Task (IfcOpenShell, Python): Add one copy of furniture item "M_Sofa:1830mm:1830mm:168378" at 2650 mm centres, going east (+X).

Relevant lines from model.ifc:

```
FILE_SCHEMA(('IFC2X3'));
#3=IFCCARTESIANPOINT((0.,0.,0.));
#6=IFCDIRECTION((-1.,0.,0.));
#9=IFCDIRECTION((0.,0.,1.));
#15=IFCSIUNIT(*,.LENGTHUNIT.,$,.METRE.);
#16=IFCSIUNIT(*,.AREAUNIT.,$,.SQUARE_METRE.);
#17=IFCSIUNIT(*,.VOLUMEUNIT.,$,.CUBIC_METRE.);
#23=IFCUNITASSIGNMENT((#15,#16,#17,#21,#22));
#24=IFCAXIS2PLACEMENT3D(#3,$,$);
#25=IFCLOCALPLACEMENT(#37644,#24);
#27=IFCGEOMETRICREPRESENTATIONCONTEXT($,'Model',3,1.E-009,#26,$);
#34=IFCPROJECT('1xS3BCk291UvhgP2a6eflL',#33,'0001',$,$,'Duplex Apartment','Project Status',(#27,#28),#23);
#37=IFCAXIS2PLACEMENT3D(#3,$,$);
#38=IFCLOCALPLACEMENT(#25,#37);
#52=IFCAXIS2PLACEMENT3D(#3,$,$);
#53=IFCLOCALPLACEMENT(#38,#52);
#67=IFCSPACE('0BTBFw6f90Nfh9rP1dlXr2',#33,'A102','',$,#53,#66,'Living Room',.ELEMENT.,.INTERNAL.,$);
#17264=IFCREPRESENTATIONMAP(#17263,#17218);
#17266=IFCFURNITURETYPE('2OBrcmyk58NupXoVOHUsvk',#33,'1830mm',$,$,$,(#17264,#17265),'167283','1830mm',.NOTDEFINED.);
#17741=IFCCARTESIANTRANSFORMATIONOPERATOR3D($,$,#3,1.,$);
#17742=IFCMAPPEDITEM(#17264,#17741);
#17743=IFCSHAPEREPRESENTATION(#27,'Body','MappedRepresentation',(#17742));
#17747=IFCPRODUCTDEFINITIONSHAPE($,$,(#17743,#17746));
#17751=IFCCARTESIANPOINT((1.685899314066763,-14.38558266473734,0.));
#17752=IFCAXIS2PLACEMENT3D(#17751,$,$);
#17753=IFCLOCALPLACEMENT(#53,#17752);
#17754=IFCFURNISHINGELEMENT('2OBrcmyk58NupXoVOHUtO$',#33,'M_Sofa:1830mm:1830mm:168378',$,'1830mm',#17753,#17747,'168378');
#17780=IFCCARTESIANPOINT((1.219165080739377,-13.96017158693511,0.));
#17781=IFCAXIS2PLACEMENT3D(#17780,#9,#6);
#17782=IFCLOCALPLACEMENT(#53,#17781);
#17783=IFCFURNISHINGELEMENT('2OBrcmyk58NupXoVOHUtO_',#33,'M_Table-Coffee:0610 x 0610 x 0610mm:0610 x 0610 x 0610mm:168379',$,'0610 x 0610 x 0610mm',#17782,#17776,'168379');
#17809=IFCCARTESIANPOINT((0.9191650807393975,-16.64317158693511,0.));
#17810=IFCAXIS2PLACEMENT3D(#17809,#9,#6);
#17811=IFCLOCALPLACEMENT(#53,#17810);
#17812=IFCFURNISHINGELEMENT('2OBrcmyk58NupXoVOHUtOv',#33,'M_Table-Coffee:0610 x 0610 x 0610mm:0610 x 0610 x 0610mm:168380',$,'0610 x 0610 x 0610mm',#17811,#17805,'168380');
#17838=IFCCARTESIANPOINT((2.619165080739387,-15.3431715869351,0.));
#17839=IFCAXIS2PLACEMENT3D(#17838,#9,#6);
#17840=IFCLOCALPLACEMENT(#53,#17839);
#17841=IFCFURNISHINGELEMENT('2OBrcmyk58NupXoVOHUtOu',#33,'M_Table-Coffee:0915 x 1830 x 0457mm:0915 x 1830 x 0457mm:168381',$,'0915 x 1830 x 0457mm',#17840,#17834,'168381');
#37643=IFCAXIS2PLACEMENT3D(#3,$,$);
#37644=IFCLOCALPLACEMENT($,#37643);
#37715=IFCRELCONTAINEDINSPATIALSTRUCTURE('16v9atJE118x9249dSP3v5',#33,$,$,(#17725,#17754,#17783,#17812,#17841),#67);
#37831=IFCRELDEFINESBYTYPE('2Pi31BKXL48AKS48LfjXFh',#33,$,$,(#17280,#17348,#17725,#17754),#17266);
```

```python
import numpy as np
import ifcopenshell
import ifcopenshell.api.geometry
import ifcopenshell.api.root
import ifcopenshell.util.element
import ifcopenshell.util.placement

model = ifcopenshell.open("model.ifc")


def reuse_history(source, copy):
    """copy_class also copies each property set's owner history, people and application; keep the originals."""
    for rel in copy.IsDefinedBy:
        if rel.is_a("IfcRelDefinesByProperties") and (history := rel.RelatingPropertyDefinition.OwnerHistory):
            rel.RelatingPropertyDefinition.OwnerHistory = source.OwnerHistory
            ifcopenshell.util.element.remove_deep2(model, history)


source = model.by_id(17754)
base = ifcopenshell.util.placement.get_local_placement(source.ObjectPlacement)
step = np.array([1.0, 0.0, 0.0]) * 2.65

for i in range(1, 2):
    copy = ifcopenshell.api.root.copy_class(model, product=source)
    copy.Representation = ifcopenshell.util.element.copy_deep(
        model, source.Representation, exclude=["IfcGeometricRepresentationContext", "IfcRepresentationMap"]
    )
    copy.Name = "M_Sofa:1830mm:1830mm"
    copy.Tag = None
    reuse_history(source, copy)
    matrix = base.copy()
    matrix[:3, 3] += i * step
    print("added at", matrix[:3, 3].round(3) + 0.0)
    ifcopenshell.api.geometry.edit_object_placement(model, product=copy, matrix=matrix, is_si=False)

model.write("model_v2.ifc")
```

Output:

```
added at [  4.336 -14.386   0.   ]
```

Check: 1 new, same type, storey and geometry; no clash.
